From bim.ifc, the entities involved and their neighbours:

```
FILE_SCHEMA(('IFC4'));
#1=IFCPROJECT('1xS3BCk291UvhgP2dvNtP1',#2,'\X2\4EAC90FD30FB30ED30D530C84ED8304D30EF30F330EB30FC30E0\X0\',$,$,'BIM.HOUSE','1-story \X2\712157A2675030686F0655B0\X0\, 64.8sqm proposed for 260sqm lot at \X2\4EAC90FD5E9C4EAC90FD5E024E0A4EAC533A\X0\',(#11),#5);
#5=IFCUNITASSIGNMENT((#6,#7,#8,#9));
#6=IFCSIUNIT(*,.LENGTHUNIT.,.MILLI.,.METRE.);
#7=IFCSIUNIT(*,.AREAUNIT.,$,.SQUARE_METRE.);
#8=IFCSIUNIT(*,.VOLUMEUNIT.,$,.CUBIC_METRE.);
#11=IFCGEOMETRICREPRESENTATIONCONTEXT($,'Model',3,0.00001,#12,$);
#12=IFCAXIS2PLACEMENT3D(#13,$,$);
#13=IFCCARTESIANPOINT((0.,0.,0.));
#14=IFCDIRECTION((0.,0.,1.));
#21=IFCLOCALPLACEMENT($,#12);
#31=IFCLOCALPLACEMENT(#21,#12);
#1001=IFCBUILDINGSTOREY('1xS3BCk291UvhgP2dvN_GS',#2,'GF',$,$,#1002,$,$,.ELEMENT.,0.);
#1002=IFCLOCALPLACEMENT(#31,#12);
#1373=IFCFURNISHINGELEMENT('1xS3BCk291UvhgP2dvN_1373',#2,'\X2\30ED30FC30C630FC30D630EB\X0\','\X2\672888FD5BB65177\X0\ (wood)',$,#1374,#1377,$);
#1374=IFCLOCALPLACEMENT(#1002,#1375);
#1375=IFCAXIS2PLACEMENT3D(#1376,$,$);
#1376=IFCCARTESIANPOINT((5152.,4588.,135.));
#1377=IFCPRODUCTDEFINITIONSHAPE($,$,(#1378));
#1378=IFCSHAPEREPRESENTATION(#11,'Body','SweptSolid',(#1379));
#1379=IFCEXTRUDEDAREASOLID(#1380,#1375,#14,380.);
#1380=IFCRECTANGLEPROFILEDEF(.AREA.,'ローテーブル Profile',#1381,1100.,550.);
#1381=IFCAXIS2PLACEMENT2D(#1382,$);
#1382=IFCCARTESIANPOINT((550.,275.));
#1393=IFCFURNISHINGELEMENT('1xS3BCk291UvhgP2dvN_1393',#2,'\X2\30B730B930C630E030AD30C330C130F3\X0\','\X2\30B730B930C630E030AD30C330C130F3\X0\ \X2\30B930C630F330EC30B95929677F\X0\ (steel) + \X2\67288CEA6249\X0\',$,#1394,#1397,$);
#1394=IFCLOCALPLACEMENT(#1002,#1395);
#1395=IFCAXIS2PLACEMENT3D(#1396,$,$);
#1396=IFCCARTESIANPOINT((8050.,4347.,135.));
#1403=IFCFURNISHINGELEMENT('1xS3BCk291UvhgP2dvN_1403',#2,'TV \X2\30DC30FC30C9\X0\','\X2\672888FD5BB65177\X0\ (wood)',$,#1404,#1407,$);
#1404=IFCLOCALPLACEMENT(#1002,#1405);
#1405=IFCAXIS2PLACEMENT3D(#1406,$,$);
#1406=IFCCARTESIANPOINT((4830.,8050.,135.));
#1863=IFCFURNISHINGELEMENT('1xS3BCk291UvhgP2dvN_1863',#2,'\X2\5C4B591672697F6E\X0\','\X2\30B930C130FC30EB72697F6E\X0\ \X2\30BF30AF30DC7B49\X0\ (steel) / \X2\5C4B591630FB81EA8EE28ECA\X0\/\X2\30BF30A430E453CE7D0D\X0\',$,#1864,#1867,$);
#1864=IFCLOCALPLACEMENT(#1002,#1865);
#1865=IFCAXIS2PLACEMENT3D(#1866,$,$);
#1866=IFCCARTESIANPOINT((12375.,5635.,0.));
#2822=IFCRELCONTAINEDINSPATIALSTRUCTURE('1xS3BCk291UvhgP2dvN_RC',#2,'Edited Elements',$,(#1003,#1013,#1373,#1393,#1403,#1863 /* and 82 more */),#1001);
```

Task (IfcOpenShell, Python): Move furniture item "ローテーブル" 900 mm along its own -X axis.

```python
import ifcopenshell
import ifcopenshell.api.geometry
import ifcopenshell.util.placement

model = ifcopenshell.open("bim.ifc")

item = model.by_guid("1xS3BCk291UvhgP2dvN_1373")
matrix = ifcopenshell.util.placement.get_local_placement(item.ObjectPlacement)
matrix[:3, 3] -= matrix[:3, 0] * 900.0
ifcopenshell.api.geometry.edit_object_placement(model, product=item, matrix=matrix, is_si=False)

print(ifcopenshell.util.placement.get_local_placement(item.ObjectPlacement).round(3) + 0.0)

model.write("bim_updated.ifc")
```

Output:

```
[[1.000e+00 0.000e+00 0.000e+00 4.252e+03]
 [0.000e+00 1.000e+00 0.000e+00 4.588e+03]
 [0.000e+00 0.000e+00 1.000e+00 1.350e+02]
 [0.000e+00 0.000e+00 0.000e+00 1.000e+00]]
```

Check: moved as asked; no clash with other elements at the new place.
